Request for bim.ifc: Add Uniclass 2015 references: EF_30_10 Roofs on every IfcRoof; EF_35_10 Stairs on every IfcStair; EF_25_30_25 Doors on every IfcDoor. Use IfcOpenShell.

First a look at what the model holds.

```python
import ifcopenshell

model = ifcopenshell.open("bim.ifc")
print(model.schema)
print("classifications:", [c.Name for c in model.by_type("IfcClassification")])
for ifc_class in ("IfcDoor", "IfcRoof", "IfcStair", "IfcWall", "IfcWindow"):
    print(ifc_class, len(model.by_type(ifc_class)))
```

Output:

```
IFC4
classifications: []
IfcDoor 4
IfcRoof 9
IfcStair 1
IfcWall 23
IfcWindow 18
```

```python
import ifcopenshell
import ifcopenshell.api.classification

model = ifcopenshell.open("bim.ifc")

system = ifcopenshell.api.classification.add_classification(model, classification="Uniclass 2015")

codes = {
    "IfcRoof": ("EF_30_10", "Roofs"),
    "IfcStair": ("EF_35_10", "Stairs"),
    "IfcDoor": ("EF_25_30_25", "Doors"),
}
for ifc_class, (code, name) in codes.items():
    products = model.by_type(ifc_class)
    ifcopenshell.api.classification.add_reference(
        model, products=products, classification=system, identification=code, name=name
    )
    print(code, len(products))

model.write("bim_rev.ifc")
```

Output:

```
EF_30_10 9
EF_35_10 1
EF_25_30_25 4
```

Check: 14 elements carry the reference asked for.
